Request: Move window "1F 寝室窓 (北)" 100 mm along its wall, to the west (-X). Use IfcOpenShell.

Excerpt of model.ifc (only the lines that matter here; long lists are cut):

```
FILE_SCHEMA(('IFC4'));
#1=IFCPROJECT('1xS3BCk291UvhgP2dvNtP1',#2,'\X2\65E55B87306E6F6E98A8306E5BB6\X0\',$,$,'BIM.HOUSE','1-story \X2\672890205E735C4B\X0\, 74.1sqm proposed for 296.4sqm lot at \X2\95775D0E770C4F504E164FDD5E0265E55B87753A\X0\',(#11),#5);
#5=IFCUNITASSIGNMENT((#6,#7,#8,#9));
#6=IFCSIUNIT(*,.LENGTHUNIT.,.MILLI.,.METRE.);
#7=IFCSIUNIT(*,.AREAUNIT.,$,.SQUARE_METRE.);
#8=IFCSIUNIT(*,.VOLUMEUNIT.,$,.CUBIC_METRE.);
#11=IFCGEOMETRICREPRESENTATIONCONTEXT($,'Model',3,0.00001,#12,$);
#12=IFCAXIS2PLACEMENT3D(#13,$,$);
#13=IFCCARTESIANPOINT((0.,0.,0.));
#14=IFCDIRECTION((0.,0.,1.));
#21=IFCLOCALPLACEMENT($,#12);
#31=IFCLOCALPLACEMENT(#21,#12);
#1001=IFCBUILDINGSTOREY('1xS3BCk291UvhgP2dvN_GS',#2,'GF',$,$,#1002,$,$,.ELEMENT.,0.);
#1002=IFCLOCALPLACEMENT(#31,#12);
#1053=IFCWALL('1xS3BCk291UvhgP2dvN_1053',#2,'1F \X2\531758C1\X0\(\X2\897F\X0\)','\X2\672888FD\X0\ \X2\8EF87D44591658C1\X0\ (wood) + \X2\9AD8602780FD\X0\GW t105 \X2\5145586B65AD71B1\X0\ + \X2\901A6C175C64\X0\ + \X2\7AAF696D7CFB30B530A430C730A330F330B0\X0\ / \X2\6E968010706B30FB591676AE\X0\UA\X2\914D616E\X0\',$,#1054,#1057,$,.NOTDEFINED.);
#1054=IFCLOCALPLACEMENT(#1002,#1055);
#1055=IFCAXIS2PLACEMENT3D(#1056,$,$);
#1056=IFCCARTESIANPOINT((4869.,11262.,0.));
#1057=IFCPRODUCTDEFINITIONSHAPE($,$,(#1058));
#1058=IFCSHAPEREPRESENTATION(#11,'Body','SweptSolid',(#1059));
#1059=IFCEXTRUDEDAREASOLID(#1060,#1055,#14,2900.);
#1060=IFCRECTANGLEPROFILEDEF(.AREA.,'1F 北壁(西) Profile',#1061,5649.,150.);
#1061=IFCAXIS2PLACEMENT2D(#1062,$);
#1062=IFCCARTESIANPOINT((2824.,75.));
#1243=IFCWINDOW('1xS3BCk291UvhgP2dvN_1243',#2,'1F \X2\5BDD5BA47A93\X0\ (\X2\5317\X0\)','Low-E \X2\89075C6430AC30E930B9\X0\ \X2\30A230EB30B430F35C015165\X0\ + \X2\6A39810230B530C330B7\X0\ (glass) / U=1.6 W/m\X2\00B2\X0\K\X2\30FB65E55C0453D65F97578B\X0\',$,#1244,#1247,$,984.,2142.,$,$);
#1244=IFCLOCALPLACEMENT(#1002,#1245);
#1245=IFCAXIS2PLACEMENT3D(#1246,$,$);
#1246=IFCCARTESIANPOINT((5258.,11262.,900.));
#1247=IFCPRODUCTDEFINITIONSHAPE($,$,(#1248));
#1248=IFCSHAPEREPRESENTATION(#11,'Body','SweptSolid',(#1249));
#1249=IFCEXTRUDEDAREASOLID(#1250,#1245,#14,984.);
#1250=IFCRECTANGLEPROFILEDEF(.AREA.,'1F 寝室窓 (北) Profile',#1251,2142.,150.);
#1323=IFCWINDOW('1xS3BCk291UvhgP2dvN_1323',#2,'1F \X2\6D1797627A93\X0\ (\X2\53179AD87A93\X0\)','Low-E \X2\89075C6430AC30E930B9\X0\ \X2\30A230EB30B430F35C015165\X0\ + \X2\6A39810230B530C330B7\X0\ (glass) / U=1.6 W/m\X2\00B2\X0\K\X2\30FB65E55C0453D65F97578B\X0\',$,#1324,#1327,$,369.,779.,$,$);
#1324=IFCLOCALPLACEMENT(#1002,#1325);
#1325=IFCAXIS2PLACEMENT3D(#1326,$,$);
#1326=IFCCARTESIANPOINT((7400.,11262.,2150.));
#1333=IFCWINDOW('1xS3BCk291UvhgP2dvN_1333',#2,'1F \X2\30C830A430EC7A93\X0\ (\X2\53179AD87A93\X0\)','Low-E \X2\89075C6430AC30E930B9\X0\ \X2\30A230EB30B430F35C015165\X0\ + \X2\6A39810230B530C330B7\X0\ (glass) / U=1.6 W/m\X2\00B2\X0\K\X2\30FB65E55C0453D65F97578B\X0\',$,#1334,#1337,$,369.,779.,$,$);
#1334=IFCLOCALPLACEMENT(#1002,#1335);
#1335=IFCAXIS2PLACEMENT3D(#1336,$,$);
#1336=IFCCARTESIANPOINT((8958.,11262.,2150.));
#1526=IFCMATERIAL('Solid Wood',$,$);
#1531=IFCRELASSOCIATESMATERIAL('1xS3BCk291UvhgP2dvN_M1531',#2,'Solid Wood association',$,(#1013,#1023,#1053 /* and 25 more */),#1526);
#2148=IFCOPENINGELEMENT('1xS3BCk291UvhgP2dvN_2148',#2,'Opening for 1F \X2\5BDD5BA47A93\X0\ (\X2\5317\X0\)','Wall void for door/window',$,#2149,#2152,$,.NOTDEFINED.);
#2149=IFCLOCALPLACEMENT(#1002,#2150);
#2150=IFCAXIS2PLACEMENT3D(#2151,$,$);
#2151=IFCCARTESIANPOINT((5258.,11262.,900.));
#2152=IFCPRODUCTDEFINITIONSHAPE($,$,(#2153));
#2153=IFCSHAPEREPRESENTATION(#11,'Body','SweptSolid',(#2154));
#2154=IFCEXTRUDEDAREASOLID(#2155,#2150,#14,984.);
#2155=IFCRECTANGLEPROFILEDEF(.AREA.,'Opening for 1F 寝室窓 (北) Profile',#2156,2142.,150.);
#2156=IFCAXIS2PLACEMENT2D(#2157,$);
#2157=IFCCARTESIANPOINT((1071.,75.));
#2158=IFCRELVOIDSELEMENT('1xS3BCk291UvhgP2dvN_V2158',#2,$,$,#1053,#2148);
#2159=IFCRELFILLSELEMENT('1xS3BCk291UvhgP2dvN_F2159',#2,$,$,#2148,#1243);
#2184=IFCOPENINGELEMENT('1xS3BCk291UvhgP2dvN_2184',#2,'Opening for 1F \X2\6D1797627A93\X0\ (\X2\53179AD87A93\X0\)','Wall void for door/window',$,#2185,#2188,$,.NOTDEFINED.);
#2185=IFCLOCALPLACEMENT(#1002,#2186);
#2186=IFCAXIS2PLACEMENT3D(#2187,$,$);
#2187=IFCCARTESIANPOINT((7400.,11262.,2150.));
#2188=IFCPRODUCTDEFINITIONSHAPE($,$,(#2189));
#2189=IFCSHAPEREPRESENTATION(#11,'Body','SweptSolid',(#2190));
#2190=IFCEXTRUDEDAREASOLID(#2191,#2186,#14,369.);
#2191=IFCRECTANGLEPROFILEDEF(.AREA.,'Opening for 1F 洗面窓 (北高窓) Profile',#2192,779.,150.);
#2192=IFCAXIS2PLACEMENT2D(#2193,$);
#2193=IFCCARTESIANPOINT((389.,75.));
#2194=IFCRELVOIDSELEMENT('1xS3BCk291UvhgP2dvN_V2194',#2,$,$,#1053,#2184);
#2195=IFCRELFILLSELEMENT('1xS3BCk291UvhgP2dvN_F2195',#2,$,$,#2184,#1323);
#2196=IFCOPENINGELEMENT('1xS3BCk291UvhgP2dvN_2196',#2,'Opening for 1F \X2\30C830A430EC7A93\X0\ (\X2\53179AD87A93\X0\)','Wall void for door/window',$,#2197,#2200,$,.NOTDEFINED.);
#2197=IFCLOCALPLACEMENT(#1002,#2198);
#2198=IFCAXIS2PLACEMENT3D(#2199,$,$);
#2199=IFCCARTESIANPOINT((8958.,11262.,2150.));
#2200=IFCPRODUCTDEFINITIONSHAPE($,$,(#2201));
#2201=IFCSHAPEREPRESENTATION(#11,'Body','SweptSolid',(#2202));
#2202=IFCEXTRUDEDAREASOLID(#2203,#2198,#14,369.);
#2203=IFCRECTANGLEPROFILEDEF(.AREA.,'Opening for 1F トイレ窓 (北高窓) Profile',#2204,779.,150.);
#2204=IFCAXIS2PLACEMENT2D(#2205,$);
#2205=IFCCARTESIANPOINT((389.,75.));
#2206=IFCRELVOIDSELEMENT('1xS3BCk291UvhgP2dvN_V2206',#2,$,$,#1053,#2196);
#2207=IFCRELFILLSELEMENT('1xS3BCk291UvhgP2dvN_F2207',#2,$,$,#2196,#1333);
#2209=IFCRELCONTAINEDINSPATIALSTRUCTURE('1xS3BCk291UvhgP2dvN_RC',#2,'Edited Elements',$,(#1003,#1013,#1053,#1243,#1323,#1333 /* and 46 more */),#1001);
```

```python
import ifcopenshell
import ifcopenshell.api.geometry
import ifcopenshell.util.placement
import ifcopenshell.util.unit

model = ifcopenshell.open("model.ifc")
unit_scale = ifcopenshell.util.unit.calculate_unit_scale(model)

window = model.by_guid("1xS3BCk291UvhgP2dvN_1243")
opening = window.FillsVoids[0].RelatingOpeningElement
wall = opening.VoidsElements[0].RelatingBuildingElement

wall_matrix = ifcopenshell.util.placement.get_local_placement(wall.ObjectPlacement)
shift = wall_matrix[:3, 0] * -0.1 / unit_scale
before = ifcopenshell.util.placement.get_local_placement(window.ObjectPlacement)[:3, 3].copy()

# The window is not placed relative to its opening, so move both.
for product in (opening, window):
    matrix = ifcopenshell.util.placement.get_local_placement(product.ObjectPlacement)
    matrix[:3, 3] += shift
    ifcopenshell.api.geometry.edit_object_placement(model, product=product, matrix=matrix, is_si=False)

after = ifcopenshell.util.placement.get_local_placement(window.ObjectPlacement)[:3, 3]
print("window moved by", (after - before).round(3) + 0.0)

model.write("model-out.ifc")
```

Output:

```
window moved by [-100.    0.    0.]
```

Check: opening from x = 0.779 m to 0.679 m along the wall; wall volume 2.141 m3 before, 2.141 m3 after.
